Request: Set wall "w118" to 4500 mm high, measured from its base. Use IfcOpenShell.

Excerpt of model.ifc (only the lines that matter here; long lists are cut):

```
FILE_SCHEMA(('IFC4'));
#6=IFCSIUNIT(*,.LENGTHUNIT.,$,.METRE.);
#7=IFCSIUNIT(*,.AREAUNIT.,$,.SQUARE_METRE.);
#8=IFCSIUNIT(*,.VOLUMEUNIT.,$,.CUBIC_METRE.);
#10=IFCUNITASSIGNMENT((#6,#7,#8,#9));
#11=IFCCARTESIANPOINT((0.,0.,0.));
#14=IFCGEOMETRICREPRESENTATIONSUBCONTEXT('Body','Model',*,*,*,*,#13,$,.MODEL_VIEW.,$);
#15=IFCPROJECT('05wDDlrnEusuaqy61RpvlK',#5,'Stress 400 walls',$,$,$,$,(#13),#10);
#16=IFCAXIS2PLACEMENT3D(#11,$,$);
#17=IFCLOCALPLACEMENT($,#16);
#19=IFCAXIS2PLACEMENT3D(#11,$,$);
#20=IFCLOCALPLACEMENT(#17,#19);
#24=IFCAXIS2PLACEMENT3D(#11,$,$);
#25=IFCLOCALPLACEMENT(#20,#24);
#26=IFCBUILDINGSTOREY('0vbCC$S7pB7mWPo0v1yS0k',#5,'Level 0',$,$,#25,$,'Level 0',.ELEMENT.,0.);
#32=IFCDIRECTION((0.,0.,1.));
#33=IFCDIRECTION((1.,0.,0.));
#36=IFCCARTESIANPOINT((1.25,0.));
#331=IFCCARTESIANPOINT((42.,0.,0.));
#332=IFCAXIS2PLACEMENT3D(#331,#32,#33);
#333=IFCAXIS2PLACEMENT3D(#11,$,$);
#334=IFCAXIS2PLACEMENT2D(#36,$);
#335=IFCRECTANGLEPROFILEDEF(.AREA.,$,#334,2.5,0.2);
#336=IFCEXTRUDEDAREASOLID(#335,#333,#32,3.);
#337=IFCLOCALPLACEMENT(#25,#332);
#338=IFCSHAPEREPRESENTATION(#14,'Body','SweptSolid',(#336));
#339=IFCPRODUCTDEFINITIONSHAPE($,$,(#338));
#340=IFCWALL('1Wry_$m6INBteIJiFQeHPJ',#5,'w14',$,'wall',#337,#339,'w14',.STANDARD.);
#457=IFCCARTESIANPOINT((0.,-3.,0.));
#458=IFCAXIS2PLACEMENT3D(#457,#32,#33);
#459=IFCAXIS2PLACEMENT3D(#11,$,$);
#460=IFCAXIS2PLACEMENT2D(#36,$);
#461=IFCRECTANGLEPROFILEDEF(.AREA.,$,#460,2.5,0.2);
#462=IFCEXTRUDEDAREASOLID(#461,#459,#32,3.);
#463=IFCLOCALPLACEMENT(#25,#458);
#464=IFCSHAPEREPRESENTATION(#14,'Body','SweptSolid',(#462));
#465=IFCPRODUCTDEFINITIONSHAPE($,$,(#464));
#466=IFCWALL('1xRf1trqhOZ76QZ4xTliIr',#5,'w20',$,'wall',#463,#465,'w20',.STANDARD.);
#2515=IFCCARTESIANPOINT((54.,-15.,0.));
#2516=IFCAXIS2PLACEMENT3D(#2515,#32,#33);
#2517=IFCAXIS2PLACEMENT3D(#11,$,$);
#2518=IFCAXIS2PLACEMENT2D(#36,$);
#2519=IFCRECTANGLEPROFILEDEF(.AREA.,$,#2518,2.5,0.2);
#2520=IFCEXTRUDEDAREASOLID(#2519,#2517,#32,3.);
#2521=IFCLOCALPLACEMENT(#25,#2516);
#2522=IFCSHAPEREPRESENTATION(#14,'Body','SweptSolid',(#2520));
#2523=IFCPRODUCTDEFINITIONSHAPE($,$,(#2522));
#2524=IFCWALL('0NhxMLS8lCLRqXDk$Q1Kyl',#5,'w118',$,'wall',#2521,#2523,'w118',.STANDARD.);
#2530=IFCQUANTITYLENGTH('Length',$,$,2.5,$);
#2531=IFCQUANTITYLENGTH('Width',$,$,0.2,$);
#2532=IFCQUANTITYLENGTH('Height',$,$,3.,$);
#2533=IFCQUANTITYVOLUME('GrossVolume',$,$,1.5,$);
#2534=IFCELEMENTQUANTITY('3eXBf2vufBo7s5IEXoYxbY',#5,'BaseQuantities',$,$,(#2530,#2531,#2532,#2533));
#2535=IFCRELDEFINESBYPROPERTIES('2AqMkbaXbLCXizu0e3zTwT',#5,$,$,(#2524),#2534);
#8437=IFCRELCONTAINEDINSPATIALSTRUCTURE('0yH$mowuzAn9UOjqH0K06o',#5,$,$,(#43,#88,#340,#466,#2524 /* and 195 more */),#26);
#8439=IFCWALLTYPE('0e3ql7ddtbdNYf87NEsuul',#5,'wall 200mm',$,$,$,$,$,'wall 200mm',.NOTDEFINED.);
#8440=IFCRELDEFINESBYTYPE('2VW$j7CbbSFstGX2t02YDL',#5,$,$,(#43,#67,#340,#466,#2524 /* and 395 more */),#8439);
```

```python
import ifcopenshell
import ifcopenshell.api.pset
import ifcopenshell.geom
import ifcopenshell.util.element
import ifcopenshell.util.representation
import ifcopenshell.util.shape
import ifcopenshell.util.unit

model = ifcopenshell.open("model.ifc")
unit_scale = ifcopenshell.util.unit.calculate_unit_scale(model)
volume_scale = ifcopenshell.util.unit.calculate_unit_scale(model, "VOLUMEUNIT")
settings = ifcopenshell.geom.settings()


def volume(element):
    """Net volume in cubic metres, openings subtracted."""
    shape = ifcopenshell.geom.create_shape(settings, element)
    return ifcopenshell.util.shape.get_volume(shape.geometry)


wall = model.by_guid("0NhxMLS8lCLRqXDk$Q1Kyl")
before = volume(wall)

body = ifcopenshell.util.representation.get_representation(wall, "Model", "Body")
solid = body.Items[0]
old_height = solid.Depth
solid.Depth = 4.5
after = volume(wall)

# Update the stored height, areas and volumes.
qto = model.by_id(ifcopenshell.util.element.get_pset(wall, "BaseQuantities", should_inherit=False)["id"])
ifcopenshell.api.pset.edit_qto(model, qto=qto, properties={
    "Height": solid.Depth,
    "GrossVolume": ifcopenshell.util.element.get_pset(wall, "BaseQuantities", "GrossVolume") * solid.Depth / old_height,
})

print(f"height {old_height:g} -> {solid.Depth:g}, volume {before:.3f} -> {after:.3f} m3")

model.write("model_updated.ifc")
```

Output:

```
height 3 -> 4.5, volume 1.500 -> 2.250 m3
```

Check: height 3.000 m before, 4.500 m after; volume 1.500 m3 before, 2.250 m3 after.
